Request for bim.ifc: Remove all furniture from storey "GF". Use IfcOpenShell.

First a look at what the model holds.

```python
import ifcopenshell
import ifcopenshell.util.element

model = ifcopenshell.open("bim.ifc")
print(model.schema)
storey = next(s for s in model.by_type("IfcBuildingStorey") if s.Name == "GF")
furniture = [e for e in ifcopenshell.util.element.get_decomposition(storey) if e.is_a("IfcFurnishingElement")]
seen = {}
for e in furniture:
    element_type = ifcopenshell.util.element.get_type(e)
    name = element_type.Name if element_type not in (None, e) else None
    seen[name] = seen.get(name, 0) + 1
for name, count in sorted(seen.items(), key=str):
    print(count, "x", name)
```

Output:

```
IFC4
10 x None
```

```python
import ifcopenshell
import ifcopenshell.api.root
import ifcopenshell.util.element

model = ifcopenshell.open("bim.ifc")

storey = next(s for s in model.by_type("IfcBuildingStorey") if s.Name == "GF")
furniture = [e for e in ifcopenshell.util.element.get_decomposition(storey) if e.is_a("IfcFurnishingElement")]

for e in furniture:
    ifcopenshell.api.root.remove_product(model, product=e)
print(len(furniture), "removed")

model.write("bim_rev.ifc")
```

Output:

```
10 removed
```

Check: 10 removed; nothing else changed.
